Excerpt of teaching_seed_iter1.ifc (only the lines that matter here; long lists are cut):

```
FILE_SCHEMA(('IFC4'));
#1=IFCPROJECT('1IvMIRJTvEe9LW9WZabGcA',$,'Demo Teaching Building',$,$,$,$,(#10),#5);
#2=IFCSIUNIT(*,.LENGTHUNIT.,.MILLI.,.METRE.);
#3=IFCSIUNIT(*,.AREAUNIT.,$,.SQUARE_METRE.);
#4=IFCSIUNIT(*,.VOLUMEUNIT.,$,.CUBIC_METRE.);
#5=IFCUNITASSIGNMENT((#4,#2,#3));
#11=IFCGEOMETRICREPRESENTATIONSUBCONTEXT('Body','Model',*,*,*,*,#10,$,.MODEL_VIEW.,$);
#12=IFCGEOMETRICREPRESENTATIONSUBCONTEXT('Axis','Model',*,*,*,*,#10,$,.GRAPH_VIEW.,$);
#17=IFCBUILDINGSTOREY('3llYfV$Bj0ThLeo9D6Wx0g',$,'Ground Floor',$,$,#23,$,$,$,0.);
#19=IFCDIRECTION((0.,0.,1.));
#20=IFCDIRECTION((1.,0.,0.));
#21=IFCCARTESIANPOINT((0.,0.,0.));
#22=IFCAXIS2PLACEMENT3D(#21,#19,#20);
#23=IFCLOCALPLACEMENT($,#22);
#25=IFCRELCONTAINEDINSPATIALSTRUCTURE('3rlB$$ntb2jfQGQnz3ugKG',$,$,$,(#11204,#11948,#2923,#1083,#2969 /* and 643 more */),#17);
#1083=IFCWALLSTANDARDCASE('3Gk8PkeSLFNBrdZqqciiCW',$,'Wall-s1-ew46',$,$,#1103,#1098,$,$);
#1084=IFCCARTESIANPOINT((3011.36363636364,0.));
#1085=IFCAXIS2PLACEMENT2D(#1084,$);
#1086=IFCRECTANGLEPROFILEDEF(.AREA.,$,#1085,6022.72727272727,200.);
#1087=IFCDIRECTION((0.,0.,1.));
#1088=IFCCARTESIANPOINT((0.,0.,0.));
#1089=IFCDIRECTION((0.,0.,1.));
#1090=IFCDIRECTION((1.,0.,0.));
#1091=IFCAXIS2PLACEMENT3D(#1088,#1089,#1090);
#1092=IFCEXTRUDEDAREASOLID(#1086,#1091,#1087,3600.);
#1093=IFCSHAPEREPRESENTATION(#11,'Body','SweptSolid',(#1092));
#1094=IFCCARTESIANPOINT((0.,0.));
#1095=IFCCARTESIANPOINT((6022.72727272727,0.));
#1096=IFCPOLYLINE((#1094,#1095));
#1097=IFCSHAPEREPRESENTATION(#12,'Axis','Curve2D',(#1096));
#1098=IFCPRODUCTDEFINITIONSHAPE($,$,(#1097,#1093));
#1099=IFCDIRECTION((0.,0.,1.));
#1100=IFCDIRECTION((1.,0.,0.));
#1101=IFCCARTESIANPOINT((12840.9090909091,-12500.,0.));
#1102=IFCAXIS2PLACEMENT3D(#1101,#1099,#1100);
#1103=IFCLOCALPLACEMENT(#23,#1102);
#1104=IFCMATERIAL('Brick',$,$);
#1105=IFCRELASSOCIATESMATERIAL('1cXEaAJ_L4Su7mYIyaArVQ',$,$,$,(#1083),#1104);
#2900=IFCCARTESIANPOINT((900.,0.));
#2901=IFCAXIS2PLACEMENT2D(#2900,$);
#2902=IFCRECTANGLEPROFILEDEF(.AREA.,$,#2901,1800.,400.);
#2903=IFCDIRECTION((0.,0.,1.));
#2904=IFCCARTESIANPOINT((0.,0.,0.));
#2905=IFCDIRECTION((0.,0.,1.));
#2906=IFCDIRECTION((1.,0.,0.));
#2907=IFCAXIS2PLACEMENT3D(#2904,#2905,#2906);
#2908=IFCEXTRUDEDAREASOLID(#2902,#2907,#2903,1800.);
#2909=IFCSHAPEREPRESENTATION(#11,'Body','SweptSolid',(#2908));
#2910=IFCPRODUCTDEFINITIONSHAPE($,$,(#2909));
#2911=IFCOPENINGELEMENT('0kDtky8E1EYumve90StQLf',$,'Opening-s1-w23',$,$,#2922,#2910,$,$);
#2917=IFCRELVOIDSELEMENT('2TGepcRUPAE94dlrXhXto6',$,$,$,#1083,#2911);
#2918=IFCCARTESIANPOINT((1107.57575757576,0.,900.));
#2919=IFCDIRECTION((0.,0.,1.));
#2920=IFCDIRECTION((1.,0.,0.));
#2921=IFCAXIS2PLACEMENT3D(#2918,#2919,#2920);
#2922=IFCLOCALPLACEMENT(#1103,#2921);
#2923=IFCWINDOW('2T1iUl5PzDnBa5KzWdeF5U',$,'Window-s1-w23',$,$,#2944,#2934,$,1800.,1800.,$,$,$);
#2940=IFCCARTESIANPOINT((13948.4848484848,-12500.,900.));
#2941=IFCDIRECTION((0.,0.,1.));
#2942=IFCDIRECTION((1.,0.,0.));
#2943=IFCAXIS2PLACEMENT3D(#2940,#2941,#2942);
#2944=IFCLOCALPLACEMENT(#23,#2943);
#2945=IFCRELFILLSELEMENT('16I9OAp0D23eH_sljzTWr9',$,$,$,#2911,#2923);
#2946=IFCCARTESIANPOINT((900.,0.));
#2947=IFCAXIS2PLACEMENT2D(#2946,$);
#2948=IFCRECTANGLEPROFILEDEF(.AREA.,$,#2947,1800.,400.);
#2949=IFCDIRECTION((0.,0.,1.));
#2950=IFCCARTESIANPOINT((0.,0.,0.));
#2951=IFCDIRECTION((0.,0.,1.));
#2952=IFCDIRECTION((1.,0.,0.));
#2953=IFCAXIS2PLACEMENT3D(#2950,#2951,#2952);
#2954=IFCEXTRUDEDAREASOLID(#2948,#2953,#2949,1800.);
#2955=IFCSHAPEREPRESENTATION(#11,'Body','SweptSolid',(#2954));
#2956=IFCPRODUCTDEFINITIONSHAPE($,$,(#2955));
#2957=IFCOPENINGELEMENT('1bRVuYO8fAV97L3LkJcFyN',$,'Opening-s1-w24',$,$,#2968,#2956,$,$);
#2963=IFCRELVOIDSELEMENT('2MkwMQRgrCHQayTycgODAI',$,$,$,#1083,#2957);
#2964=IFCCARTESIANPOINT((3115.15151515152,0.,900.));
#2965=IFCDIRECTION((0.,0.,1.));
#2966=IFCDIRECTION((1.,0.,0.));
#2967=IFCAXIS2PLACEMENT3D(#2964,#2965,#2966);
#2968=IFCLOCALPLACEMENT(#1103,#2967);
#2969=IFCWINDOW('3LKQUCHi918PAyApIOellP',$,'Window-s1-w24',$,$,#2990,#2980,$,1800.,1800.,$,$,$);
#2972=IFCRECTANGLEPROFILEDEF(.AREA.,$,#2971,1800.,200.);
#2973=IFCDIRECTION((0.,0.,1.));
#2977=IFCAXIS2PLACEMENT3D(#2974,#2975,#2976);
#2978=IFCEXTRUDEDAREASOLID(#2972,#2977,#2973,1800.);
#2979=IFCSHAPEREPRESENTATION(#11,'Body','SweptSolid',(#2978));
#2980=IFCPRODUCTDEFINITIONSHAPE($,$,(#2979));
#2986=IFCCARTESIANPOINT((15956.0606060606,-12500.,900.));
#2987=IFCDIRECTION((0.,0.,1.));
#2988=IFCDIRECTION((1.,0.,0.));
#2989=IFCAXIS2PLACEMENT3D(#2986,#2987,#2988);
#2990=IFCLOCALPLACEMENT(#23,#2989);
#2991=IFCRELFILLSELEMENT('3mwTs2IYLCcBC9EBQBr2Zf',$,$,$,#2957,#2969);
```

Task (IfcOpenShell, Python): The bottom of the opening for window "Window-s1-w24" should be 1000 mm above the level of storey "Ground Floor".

```python
import numpy as np
import ifcopenshell
import ifcopenshell.api.geometry
import ifcopenshell.geom
import ifcopenshell.util.element
import ifcopenshell.util.placement
import ifcopenshell.util.shape
import ifcopenshell.util.unit

model = ifcopenshell.open("teaching_seed_iter1.ifc")
unit_scale = ifcopenshell.util.unit.calculate_unit_scale(model)

window = model.by_guid("3LKQUCHi918PAyApIOellP")
opening = window.FillsVoids[0].RelatingOpeningElement
storey = ifcopenshell.util.element.get_container(window, ifc_class="IfcBuildingStorey")
level = ifcopenshell.util.placement.get_local_placement(storey.ObjectPlacement)[2, 3]

# The opening's origin need not be at the sill, so measure its lowest point.
shape = ifcopenshell.geom.create_shape(ifcopenshell.geom.settings(), opening)
bottom = ifcopenshell.util.shape.get_shape_bottom_elevation(shape, shape.geometry) / unit_scale
dz = level + 1 / unit_scale - bottom

shift = np.array([0.0, 0.0, dz])
# The window is not placed relative to its opening, so move both.
for product in (opening, window):
    matrix = ifcopenshell.util.placement.get_local_placement(product.ObjectPlacement)
    matrix[:3, 3] += shift
    ifcopenshell.api.geometry.edit_object_placement(model, product=product, matrix=matrix, is_si=False)

print(f"moved by {dz * unit_scale:+.3f} m")

model.write("teaching_seed_iter1_rev.ifc")
```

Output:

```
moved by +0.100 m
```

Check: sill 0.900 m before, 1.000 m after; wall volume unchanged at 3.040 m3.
